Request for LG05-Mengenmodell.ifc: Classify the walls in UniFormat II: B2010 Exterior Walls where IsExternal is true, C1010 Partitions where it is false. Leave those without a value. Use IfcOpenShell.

First a look at what the model holds.

```python
import ifcopenshell
import ifcopenshell.util.element

model = ifcopenshell.open("LG05-Mengenmodell.ifc")
print(model.schema)
print("classifications:", [c.Name for c in model.by_type("IfcClassification")])
values = [ifcopenshell.util.element.get_pset(e, "Pset_WallCommon", "IsExternal") for e in model.by_type("IfcWall")]
for value in (True, False, None):
    print("IsExternal", value, values.count(value))
```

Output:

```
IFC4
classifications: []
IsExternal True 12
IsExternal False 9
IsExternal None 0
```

```python
import ifcopenshell
import ifcopenshell.api.classification
import ifcopenshell.util.element

model = ifcopenshell.open("LG05-Mengenmodell.ifc")

system = ifcopenshell.api.classification.add_classification(model, classification="UniFormat II")

walls = model.by_type("IfcWall")
external = {e: ifcopenshell.util.element.get_pset(e, "Pset_WallCommon", "IsExternal") for e in walls}
for flag, code, name in ((True, "B2010", "Exterior Walls"), (False, "C1010", "Partitions")):
    products = [e for e in walls if external[e] is flag]
    ifcopenshell.api.classification.add_reference(
        model, products=products, classification=system, identification=code, name=name
    )
    print(code, len(products))

model.write("LG05-Mengenmodell_updated.ifc")
```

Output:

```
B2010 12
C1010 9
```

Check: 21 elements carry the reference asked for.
